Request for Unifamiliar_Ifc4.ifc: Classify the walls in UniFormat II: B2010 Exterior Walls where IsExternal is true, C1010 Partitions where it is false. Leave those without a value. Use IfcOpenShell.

First a look at what the model holds.

```python
import ifcopenshell
import ifcopenshell.util.element

model = ifcopenshell.open("Unifamiliar_Ifc4.ifc")
print(model.schema)
print("classifications:", [c.Name for c in model.by_type("IfcClassification")])
values = [ifcopenshell.util.element.get_pset(e, "Pset_WallCommon", "IsExternal") for e in model.by_type("IfcWall")]
for value in (True, False, None):
    print("IsExternal", value, values.count(value))
```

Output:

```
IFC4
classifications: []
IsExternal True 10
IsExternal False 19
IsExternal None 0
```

```python
import ifcopenshell
import ifcopenshell.api.classification
import ifcopenshell.util.element

model = ifcopenshell.open("Unifamiliar_Ifc4.ifc")

system = ifcopenshell.api.classification.add_classification(model, classification="UniFormat II")

walls = model.by_type("IfcWall")
external = {e: ifcopenshell.util.element.get_pset(e, "Pset_WallCommon", "IsExternal") for e in walls}
for flag, code, name in ((True, "B2010", "Exterior Walls"), (False, "C1010", "Partitions")):
    products = [e for e in walls if external[e] is flag]
    ifcopenshell.api.classification.add_reference(
        model, products=products, classification=system, identification=code, name=name
    )
    print(code, len(products))

model.write("Unifamiliar_Ifc4_edited.ifc")
```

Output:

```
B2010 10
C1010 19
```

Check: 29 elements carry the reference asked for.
